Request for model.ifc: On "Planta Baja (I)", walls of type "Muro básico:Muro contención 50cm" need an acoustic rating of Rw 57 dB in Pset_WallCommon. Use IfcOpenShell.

First a look at what the model holds.

```python
import ifcopenshell
import ifcopenshell.util.element

model = ifcopenshell.open("model.ifc")
print(model.schema)
storey = next(s for s in model.by_type("IfcBuildingStorey") if s.Name == "Planta Baja (I)")
walls = [e for e in ifcopenshell.util.element.get_decomposition(storey) if e.is_a("IfcWall")]
seen = {}
for e in walls:
    element_type = ifcopenshell.util.element.get_type(e)
    key = (element_type.Name if element_type != e and element_type else None, ifcopenshell.util.element.get_pset(e, "Pset_WallCommon", "AcousticRating"))
    seen[key] = seen.get(key, 0) + 1
for (name, value), count in sorted(seen.items(), key=str):
    print(count, "x", name, "|", value)
```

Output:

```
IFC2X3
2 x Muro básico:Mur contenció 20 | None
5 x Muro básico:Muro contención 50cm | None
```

```python
import ifcopenshell
import ifcopenshell.api.pset
import ifcopenshell.util.element

model = ifcopenshell.open("model.ifc")

storey = next(s for s in model.by_type("IfcBuildingStorey") if s.Name == "Planta Baja (I)")
walls = [e for e in ifcopenshell.util.element.get_decomposition(storey) if e.is_a("IfcWall")]

count = 0
for e in walls:
    element_type = ifcopenshell.util.element.get_type(e)
    if element_type in (None, e) or element_type.Name != "Muro básico:Muro contención 50cm":
        continue
    # add_pset returns the element's existing set when there is one.
    pset = ifcopenshell.api.pset.add_pset(model, product=e, name="Pset_WallCommon")
    ifcopenshell.api.pset.edit_pset(model, pset=pset, properties={"AcousticRating": "Rw 57 dB"})
    count += 1

print(count, "walls updated")

model.write("model_edited.ifc")
```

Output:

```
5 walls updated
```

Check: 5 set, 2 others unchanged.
